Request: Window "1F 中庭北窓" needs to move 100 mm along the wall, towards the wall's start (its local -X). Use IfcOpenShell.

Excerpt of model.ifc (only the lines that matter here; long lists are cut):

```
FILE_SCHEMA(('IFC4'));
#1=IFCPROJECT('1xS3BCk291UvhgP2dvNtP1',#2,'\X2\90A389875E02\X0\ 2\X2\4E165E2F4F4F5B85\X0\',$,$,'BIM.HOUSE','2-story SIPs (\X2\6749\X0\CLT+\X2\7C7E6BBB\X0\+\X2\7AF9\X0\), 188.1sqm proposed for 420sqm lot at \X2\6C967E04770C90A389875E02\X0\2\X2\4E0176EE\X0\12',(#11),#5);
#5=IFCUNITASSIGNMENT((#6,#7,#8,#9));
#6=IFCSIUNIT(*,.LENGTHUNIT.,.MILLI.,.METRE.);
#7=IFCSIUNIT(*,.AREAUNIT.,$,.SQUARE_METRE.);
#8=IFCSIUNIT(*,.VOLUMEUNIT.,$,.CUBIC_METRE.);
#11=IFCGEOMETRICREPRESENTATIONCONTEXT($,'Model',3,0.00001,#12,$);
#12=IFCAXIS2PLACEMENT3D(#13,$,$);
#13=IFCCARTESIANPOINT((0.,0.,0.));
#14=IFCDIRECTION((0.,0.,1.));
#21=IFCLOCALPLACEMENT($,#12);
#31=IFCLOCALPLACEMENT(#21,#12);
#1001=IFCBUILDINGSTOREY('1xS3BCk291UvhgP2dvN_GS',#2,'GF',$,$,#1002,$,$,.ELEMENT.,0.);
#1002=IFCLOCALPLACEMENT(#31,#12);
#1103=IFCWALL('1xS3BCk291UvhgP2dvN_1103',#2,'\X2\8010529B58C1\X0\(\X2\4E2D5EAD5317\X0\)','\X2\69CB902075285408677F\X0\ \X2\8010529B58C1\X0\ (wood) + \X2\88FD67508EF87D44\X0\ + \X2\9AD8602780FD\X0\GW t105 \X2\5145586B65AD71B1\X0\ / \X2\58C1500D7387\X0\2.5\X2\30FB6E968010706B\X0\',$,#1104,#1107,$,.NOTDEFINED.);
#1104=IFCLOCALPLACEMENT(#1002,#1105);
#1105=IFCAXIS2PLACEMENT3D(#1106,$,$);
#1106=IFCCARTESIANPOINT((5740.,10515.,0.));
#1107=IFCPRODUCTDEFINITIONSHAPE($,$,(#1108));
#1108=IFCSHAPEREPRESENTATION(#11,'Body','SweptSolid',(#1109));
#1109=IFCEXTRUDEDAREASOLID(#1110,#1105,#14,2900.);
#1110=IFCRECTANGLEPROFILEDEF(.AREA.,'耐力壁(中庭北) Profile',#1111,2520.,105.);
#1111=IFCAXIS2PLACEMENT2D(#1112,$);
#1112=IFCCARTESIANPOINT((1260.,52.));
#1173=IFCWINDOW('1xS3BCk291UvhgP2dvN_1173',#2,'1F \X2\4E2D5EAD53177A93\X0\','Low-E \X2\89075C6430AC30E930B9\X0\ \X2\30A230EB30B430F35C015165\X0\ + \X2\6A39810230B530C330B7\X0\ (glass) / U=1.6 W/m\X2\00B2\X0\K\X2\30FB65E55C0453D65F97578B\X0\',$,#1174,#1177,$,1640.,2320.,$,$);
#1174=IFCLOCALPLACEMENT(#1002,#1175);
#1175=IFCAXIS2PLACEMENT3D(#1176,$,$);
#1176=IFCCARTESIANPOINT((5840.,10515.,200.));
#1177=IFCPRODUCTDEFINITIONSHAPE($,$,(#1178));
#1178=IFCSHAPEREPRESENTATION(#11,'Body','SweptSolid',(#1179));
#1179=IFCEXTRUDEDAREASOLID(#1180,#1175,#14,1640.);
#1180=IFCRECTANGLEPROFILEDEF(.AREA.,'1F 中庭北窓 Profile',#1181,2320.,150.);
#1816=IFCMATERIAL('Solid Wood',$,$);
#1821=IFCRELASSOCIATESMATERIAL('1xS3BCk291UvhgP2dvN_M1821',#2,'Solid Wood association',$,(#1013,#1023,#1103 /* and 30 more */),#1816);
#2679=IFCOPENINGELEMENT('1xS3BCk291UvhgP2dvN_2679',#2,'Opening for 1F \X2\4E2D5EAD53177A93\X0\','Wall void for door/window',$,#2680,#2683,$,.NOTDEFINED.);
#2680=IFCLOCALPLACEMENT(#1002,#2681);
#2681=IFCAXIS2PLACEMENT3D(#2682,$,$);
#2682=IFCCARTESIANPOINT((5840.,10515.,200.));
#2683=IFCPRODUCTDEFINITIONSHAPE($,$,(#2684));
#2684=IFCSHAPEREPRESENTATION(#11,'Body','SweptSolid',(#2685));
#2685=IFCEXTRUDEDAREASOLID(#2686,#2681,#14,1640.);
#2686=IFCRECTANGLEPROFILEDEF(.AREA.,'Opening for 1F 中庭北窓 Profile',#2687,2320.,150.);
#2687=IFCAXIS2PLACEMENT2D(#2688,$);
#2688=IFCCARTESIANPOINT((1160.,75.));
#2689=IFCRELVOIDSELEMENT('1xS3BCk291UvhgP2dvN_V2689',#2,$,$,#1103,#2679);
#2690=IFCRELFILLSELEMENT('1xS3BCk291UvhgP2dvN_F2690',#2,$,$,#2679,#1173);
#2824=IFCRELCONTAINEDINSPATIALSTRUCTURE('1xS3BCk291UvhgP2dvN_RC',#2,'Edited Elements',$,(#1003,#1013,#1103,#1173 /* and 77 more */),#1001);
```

```python
import ifcopenshell
import ifcopenshell.api.geometry
import ifcopenshell.util.placement
import ifcopenshell.util.unit

model = ifcopenshell.open("model.ifc")
unit_scale = ifcopenshell.util.unit.calculate_unit_scale(model)

window = model.by_id(1173)
opening = window.FillsVoids[0].RelatingOpeningElement
wall = opening.VoidsElements[0].RelatingBuildingElement

wall_matrix = ifcopenshell.util.placement.get_local_placement(wall.ObjectPlacement)
shift = wall_matrix[:3, 0] * -0.1 / unit_scale
before = ifcopenshell.util.placement.get_local_placement(window.ObjectPlacement)[:3, 3].copy()

# The window is not placed relative to its opening, so move both.
for product in (opening, window):
    matrix = ifcopenshell.util.placement.get_local_placement(product.ObjectPlacement)
    matrix[:3, 3] += shift
    ifcopenshell.api.geometry.edit_object_placement(model, product=product, matrix=matrix, is_si=False)

after = ifcopenshell.util.placement.get_local_placement(window.ObjectPlacement)[:3, 3]
print("window moved by", (after - before).round(3) + 0.0)

model.write("model_updated.ifc")
```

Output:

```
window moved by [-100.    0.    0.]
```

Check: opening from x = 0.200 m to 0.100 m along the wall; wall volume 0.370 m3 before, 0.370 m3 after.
